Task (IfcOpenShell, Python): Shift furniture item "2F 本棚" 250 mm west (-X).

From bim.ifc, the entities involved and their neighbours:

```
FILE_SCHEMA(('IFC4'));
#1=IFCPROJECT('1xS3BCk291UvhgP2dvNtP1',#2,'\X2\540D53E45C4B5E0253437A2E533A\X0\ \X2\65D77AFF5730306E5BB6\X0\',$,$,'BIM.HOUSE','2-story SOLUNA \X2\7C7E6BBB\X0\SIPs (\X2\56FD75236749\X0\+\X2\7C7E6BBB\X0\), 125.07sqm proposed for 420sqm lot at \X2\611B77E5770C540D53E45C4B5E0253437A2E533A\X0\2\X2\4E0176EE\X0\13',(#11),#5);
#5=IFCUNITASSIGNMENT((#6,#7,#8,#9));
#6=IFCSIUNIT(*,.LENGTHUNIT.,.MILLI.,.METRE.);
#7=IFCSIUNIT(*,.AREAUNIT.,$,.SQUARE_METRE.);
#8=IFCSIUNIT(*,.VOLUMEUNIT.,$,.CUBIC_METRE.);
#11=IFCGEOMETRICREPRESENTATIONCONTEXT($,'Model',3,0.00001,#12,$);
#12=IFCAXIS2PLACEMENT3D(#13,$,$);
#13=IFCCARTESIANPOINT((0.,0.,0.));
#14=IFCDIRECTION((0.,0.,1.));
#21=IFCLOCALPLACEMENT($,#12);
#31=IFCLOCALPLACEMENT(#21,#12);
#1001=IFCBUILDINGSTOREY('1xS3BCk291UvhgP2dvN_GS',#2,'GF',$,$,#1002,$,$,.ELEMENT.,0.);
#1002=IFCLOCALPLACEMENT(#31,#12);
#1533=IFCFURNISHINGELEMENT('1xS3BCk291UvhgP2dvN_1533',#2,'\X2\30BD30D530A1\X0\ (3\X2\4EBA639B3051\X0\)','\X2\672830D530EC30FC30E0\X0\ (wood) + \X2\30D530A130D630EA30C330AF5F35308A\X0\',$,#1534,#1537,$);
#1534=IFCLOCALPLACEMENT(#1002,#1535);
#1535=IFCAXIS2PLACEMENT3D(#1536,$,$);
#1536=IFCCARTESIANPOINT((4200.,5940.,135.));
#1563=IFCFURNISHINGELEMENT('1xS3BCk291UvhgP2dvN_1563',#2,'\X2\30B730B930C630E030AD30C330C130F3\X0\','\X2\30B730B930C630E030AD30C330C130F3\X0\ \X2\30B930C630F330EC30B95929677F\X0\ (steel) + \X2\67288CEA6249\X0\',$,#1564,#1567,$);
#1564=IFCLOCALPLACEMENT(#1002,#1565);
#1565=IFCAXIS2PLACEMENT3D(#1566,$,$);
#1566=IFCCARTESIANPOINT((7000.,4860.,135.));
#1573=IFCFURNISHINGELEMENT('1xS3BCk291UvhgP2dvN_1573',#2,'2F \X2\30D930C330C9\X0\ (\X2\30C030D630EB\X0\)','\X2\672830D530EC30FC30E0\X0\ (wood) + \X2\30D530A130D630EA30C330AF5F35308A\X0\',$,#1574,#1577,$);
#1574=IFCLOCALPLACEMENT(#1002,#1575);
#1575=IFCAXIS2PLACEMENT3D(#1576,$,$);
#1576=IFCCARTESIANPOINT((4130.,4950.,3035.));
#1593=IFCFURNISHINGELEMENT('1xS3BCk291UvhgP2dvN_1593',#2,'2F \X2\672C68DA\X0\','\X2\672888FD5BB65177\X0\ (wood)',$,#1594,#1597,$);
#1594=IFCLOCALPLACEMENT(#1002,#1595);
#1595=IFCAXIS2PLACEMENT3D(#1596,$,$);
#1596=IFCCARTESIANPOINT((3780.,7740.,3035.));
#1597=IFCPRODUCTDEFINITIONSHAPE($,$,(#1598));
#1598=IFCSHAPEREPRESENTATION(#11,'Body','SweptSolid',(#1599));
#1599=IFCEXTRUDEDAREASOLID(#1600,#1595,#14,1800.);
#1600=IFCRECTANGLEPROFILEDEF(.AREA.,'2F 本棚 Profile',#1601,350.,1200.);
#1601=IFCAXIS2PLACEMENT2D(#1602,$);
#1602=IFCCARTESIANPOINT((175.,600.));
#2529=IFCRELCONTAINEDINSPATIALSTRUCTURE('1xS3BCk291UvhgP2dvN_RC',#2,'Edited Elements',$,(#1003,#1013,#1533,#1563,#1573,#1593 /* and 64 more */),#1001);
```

```python
import ifcopenshell
import ifcopenshell.api.geometry
import ifcopenshell.util.placement

model = ifcopenshell.open("bim.ifc")

item = model.by_id(1593)
matrix = ifcopenshell.util.placement.get_local_placement(item.ObjectPlacement)
matrix[0, 3] -= 250.0
ifcopenshell.api.geometry.edit_object_placement(model, product=item, matrix=matrix, is_si=False)

print(ifcopenshell.util.placement.get_local_placement(item.ObjectPlacement).round(3) + 0.0)

model.write("bim-out.ifc")
```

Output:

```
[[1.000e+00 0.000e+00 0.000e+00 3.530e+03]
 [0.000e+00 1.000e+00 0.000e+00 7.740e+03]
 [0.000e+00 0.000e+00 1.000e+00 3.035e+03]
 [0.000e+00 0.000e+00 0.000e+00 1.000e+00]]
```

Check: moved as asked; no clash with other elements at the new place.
